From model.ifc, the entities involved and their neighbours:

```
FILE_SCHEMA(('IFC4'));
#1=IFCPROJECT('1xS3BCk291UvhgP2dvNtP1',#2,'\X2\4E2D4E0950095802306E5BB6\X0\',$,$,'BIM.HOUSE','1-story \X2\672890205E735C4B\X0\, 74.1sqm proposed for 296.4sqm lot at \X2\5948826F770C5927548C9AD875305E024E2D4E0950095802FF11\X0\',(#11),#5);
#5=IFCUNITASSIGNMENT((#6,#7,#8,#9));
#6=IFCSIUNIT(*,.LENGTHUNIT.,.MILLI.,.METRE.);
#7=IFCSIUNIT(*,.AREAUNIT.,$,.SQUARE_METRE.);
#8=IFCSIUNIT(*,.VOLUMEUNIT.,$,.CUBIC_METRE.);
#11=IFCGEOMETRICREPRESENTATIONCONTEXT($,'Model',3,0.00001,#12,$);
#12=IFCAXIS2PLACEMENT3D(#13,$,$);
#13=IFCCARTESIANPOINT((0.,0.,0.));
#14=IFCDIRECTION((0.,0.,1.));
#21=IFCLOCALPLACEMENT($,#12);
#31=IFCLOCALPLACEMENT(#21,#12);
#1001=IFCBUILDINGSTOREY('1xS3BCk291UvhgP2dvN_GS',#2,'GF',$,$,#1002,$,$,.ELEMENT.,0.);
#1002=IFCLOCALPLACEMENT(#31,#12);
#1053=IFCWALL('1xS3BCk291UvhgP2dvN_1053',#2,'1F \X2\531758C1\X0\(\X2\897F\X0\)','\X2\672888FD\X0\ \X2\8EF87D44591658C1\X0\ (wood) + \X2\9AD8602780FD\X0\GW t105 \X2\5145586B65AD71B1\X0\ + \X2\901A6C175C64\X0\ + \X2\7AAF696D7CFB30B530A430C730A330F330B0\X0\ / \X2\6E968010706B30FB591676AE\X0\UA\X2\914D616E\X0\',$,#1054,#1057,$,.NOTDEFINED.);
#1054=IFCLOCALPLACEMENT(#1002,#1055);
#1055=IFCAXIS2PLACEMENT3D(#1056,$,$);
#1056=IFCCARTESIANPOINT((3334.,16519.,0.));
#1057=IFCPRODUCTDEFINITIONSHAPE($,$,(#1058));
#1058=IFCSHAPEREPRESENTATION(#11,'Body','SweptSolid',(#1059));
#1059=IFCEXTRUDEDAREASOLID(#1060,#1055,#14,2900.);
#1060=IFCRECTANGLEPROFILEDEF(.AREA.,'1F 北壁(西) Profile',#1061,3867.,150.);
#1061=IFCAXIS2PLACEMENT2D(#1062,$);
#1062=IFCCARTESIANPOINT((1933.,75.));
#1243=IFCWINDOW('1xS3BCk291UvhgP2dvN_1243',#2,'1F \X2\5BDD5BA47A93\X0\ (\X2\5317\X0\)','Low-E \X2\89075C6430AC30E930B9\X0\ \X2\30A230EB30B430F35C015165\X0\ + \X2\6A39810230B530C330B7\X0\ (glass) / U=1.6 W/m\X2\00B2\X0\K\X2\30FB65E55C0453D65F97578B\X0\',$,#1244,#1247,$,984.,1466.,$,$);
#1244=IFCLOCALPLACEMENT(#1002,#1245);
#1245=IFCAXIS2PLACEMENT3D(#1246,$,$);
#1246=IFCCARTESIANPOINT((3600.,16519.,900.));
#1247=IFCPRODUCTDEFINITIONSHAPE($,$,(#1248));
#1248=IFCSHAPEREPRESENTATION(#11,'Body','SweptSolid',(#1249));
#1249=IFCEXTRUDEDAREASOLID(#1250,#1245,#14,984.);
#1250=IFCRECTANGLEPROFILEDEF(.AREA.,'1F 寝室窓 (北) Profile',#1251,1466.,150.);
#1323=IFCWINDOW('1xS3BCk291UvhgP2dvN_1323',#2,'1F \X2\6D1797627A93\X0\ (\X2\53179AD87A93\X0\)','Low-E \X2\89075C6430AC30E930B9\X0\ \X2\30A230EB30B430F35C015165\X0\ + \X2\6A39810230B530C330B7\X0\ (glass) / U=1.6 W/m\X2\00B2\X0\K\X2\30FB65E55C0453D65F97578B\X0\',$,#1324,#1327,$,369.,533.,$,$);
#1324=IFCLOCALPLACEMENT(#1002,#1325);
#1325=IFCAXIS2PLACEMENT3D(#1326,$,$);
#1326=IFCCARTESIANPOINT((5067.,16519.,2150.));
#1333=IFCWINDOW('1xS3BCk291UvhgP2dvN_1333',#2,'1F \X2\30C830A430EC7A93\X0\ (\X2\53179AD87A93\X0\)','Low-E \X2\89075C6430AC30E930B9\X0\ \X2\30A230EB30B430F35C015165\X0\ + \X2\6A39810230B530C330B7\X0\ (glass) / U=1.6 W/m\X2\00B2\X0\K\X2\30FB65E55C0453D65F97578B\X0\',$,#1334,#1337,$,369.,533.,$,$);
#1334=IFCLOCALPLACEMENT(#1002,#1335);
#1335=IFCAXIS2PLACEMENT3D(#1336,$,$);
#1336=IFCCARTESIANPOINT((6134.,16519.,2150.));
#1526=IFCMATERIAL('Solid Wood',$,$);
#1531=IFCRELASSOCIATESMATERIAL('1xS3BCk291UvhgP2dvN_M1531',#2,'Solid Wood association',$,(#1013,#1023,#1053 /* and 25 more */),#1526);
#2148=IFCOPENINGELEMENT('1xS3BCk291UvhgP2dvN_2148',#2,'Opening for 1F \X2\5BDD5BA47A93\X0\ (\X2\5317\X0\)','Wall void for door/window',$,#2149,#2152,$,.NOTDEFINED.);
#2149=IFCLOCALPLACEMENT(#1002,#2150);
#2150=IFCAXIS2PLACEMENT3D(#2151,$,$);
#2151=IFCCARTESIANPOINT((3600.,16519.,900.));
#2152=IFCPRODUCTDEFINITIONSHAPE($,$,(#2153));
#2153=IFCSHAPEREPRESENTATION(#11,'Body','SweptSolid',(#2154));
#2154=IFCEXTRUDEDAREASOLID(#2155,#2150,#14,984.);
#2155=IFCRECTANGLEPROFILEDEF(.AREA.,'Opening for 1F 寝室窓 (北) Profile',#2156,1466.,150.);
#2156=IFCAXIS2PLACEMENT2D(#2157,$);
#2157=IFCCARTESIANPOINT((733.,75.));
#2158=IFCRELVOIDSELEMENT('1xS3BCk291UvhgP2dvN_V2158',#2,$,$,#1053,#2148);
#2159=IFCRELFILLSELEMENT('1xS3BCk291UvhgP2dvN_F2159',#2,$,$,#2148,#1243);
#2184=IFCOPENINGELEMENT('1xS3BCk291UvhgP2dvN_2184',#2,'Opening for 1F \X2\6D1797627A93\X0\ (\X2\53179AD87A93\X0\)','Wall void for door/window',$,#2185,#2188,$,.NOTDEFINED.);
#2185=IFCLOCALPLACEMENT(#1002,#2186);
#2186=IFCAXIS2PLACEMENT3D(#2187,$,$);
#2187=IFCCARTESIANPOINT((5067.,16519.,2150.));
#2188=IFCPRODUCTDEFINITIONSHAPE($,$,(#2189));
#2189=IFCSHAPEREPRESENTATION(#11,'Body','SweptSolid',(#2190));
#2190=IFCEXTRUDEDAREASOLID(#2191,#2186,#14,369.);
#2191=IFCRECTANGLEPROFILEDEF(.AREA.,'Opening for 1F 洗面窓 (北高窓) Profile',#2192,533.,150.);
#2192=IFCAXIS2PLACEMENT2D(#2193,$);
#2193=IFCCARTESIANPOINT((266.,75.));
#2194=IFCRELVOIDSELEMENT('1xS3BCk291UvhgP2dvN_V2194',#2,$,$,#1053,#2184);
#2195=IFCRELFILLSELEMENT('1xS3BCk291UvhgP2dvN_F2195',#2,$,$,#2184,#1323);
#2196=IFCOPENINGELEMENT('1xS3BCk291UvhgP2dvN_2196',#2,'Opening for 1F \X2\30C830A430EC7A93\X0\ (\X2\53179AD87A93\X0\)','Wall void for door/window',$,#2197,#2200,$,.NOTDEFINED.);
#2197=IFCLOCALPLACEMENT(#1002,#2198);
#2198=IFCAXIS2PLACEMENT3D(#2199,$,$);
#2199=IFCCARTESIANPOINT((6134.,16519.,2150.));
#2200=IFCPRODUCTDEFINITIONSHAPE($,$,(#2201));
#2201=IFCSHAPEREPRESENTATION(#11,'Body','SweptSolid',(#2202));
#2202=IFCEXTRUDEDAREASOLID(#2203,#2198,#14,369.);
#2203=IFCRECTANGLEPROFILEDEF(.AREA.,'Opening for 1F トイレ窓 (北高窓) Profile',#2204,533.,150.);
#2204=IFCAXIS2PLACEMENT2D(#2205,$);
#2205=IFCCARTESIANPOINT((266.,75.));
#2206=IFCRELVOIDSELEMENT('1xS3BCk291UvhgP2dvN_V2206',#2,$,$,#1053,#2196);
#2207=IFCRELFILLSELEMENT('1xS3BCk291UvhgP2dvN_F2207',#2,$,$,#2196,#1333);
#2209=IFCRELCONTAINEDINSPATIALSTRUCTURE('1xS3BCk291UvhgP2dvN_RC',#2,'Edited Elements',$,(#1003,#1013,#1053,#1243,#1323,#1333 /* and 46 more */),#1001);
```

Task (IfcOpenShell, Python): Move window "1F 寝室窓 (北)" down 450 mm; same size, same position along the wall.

```python
import numpy as np
import ifcopenshell
import ifcopenshell.api.geometry
import ifcopenshell.util.placement
import ifcopenshell.util.unit

model = ifcopenshell.open("model.ifc")
unit_scale = ifcopenshell.util.unit.calculate_unit_scale(model)

window = model.by_id(1243)
opening = window.FillsVoids[0].RelatingOpeningElement
dz = -450.0

shift = np.array([0.0, 0.0, dz])
# The window is not placed relative to its opening, so move both.
for product in (opening, window):
    matrix = ifcopenshell.util.placement.get_local_placement(product.ObjectPlacement)
    matrix[:3, 3] += shift
    ifcopenshell.api.geometry.edit_object_placement(model, product=product, matrix=matrix, is_si=False)

print(f"moved by {dz * unit_scale:+.3f} m")

model.write("model_updated.ifc")
```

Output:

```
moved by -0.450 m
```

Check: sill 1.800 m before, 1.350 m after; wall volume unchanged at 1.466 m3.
